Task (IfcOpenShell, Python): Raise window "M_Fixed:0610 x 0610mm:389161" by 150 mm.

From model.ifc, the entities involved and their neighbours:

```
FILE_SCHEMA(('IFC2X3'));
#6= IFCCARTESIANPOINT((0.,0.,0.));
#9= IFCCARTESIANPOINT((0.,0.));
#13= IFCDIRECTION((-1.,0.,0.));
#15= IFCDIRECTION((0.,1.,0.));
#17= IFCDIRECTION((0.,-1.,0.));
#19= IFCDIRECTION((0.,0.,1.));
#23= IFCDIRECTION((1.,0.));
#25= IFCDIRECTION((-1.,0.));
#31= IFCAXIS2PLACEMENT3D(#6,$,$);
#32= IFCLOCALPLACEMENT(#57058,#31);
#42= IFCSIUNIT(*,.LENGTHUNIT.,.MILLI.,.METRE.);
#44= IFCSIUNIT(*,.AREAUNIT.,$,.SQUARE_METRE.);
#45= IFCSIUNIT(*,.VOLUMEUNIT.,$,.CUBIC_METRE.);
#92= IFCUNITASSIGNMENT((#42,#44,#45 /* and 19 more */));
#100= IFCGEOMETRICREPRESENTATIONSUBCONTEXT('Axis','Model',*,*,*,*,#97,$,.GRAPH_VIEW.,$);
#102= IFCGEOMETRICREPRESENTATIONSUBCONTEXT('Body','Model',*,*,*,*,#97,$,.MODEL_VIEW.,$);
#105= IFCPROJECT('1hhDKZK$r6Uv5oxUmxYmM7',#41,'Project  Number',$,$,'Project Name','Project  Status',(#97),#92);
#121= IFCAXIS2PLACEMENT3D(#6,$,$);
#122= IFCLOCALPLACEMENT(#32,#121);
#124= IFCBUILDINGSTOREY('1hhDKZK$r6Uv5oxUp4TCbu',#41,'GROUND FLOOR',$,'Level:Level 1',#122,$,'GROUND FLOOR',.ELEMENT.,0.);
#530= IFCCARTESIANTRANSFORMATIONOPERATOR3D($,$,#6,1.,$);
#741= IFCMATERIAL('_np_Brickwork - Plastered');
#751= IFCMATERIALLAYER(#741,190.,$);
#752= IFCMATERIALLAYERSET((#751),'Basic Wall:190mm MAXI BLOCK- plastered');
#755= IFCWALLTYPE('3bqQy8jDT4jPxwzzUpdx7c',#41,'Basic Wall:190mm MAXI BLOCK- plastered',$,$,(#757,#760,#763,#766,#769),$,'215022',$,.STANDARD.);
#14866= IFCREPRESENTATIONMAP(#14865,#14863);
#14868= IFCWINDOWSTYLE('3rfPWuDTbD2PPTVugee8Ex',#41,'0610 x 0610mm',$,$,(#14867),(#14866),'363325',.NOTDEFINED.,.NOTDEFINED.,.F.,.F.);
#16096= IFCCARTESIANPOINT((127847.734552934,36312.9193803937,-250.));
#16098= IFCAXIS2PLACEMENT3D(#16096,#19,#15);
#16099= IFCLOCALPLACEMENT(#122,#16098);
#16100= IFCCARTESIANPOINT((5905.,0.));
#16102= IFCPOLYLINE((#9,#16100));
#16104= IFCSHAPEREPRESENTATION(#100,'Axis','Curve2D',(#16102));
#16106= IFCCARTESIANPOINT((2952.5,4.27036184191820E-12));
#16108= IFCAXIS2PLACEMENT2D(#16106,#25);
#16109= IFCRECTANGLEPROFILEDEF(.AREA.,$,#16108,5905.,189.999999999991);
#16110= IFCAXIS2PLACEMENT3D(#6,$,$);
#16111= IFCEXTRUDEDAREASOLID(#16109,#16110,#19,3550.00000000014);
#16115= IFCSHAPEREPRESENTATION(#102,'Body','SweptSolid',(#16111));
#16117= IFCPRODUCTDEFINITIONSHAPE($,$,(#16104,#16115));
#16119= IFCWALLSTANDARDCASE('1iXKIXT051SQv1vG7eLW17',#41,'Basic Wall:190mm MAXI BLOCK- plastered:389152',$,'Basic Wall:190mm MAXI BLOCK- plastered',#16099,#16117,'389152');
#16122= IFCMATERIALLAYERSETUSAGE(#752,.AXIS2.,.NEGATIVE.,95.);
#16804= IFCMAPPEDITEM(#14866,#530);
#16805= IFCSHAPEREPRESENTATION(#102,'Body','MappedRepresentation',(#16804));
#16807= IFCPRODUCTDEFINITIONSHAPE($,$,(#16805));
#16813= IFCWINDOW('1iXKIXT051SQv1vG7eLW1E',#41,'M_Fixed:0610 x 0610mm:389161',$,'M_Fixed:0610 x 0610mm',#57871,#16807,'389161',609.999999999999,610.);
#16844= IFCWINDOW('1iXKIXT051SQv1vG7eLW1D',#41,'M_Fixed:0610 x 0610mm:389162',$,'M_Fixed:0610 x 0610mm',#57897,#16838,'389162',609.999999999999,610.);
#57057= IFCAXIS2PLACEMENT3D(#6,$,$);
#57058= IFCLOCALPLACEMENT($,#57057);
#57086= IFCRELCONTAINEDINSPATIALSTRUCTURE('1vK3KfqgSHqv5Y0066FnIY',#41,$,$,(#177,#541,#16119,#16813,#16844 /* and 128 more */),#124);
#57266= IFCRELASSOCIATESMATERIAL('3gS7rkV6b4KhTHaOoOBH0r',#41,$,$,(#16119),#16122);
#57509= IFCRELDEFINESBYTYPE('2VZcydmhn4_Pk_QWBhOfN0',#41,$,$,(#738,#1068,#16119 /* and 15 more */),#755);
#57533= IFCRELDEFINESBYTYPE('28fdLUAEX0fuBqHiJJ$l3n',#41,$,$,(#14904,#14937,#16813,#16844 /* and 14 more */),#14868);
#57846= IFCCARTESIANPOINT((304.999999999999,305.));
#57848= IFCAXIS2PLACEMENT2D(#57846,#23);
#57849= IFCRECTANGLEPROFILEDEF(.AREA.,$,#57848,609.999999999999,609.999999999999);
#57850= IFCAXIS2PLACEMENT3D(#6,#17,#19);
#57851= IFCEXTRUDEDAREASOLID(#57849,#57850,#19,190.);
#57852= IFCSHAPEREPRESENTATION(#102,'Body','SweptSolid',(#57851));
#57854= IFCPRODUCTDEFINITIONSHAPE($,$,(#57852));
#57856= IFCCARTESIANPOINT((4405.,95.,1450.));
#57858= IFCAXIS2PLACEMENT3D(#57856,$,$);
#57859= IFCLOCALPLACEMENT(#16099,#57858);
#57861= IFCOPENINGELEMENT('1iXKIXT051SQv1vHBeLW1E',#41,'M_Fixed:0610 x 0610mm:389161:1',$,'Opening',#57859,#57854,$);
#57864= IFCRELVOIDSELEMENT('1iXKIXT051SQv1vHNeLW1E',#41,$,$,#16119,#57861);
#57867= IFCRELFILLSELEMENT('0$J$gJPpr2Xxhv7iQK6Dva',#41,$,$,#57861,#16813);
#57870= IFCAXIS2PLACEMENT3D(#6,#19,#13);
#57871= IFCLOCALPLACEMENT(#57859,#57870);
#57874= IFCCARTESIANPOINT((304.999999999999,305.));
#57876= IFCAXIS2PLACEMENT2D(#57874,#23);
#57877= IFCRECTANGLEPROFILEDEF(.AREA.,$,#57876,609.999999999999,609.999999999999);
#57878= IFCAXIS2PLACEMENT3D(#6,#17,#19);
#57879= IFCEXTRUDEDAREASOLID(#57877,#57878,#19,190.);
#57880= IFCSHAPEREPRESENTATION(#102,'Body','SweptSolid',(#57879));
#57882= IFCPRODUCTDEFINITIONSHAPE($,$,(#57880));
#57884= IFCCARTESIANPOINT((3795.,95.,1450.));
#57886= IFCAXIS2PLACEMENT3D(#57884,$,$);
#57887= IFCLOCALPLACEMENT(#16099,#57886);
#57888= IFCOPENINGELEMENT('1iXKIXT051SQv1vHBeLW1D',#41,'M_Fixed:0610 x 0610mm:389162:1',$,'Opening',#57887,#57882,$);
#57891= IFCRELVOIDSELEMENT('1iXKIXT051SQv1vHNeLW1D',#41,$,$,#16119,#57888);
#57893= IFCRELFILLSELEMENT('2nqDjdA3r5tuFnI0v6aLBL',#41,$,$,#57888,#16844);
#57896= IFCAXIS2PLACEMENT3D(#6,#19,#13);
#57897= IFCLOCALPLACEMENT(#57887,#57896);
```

```python
import numpy as np
import ifcopenshell
import ifcopenshell.api.geometry
import ifcopenshell.util.placement
import ifcopenshell.util.unit

model = ifcopenshell.open("model.ifc")
unit_scale = ifcopenshell.util.unit.calculate_unit_scale(model)

window = model.by_guid("1iXKIXT051SQv1vG7eLW1E")
opening = window.FillsVoids[0].RelatingOpeningElement
dz = 0.15 / unit_scale

shift = np.array([0.0, 0.0, dz])
# The window is placed relative to its opening, so it follows when the opening moves.
matrix = ifcopenshell.util.placement.get_local_placement(opening.ObjectPlacement)
matrix[:3, 3] += shift
ifcopenshell.api.geometry.edit_object_placement(
    model, product=opening, matrix=matrix, is_si=False, should_transform_children=True
)

print(f"moved by {dz * unit_scale:+.3f} m")

model.write("model_updated.ifc")
```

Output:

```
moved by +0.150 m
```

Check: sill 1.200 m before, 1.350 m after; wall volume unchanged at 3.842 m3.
